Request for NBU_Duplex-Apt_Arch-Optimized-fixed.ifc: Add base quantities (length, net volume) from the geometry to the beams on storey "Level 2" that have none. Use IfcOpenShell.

First a look at what the model holds.

```python
import ifcopenshell
import ifcopenshell.util.element
import ifcopenshell.util.unit

model = ifcopenshell.open("NBU_Duplex-Apt_Arch-Optimized-fixed.ifc")
print(model.schema)
for unit_type in ("LENGTHUNIT", "AREAUNIT", "VOLUMEUNIT"):
    print(unit_type, ifcopenshell.util.unit.calculate_unit_scale(model, unit_type))
storey = next(s for s in model.by_type("IfcBuildingStorey") if s.Name == "Level 2")
beams = [e for e in ifcopenshell.util.element.get_decomposition(storey) if e.is_a("IfcBeam")]
for e in sorted(beams, key=lambda e: e.id()):
    print(e.id(), e.is_a(), e.Name, list(ifcopenshell.util.element.get_psets(e, qtos_only=True)), sep=" | ")
```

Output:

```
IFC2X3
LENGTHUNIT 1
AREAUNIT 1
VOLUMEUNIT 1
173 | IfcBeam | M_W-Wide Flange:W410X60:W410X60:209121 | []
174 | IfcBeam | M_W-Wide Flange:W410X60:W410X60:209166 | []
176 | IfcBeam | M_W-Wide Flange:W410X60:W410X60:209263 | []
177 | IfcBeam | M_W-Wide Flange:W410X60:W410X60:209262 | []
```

```python
import ifcopenshell
import ifcopenshell.api.pset
import ifcopenshell.geom
import ifcopenshell.util.element
import ifcopenshell.util.shape
import ifcopenshell.util.unit

model = ifcopenshell.open("NBU_Duplex-Apt_Arch-Optimized-fixed.ifc")
unit_scale = ifcopenshell.util.unit.calculate_unit_scale(model)
volume_scale = ifcopenshell.util.unit.calculate_unit_scale(model, "VOLUMEUNIT")
settings = ifcopenshell.geom.settings()

storey = next(s for s in model.by_type("IfcBuildingStorey") if s.Name == "Level 2")
beams = [e for e in ifcopenshell.util.element.get_decomposition(storey) if e.is_a("IfcBeam")]

for e in sorted(beams, key=lambda e: e.id()):
    if ifcopenshell.util.element.get_psets(e, qtos_only=True, should_inherit=False):
        continue
    # Geometry comes back in metres, in the element's own axes.
    shape = ifcopenshell.geom.create_shape(settings, e)
    values = {
        "Length": ifcopenshell.util.shape.get_max_xyz(shape.geometry) / unit_scale,
        "NetVolume": ifcopenshell.util.shape.get_volume(shape.geometry) / volume_scale,
    }
    qto = ifcopenshell.api.pset.add_qto(model, product=e, name="BaseQuantities")
    ifcopenshell.api.pset.edit_qto(model, qto=qto, properties=values)
    print(e.id(), {k: round(v, 3) for k, v in values.items()})

model.write("NBU_Duplex-Apt_Arch-Optimized-fixed_v2.ifc")
```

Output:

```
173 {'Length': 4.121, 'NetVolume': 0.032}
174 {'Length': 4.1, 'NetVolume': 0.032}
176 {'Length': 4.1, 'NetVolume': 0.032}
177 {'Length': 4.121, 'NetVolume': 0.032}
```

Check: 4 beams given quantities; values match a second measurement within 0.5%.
